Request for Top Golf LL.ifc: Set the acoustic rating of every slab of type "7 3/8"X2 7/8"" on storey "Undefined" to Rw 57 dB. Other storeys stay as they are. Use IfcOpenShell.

First a look at what the model holds.

```python
import ifcopenshell
import ifcopenshell.util.element

model = ifcopenshell.open("Top Golf LL.ifc")
print(model.schema)
storey = next(s for s in model.by_type("IfcBuildingStorey") if s.Name == "Undefined")
slabs = [e for e in ifcopenshell.util.element.get_decomposition(storey) if e.is_a("IfcSlab")]
seen = {}
for e in slabs:
    element_type = ifcopenshell.util.element.get_type(e)
    key = (element_type.Name if element_type != e and element_type else None, ifcopenshell.util.element.get_pset(e, "Pset_SlabCommon", "AcousticRating"))
    seen[key] = seen.get(key, 0) + 1
for (name, value), count in sorted(seen.items(), key=str):
    print(count, "x", name, "|", value)
```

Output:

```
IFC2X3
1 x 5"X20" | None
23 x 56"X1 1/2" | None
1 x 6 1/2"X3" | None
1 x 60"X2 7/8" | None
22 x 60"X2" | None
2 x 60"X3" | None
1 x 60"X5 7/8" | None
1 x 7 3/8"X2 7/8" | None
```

```python
import ifcopenshell
import ifcopenshell.api.pset
import ifcopenshell.util.element

model = ifcopenshell.open("Top Golf LL.ifc")

storey = next(s for s in model.by_type("IfcBuildingStorey") if s.Name == "Undefined")
slabs = [e for e in ifcopenshell.util.element.get_decomposition(storey) if e.is_a("IfcSlab")]

count = 0
for e in slabs:
    element_type = ifcopenshell.util.element.get_type(e)
    if element_type in (None, e) or element_type.Name != '7 3/8"X2 7/8"':
        continue
    # add_pset returns the element's existing set when there is one.
    pset = ifcopenshell.api.pset.add_pset(model, product=e, name="Pset_SlabCommon")
    ifcopenshell.api.pset.edit_pset(model, pset=pset, properties={"AcousticRating": "Rw 57 dB"})
    count += 1

print(count, "slabs updated")

model.write("Top Golf LL_edited.ifc")
```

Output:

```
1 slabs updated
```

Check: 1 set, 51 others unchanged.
